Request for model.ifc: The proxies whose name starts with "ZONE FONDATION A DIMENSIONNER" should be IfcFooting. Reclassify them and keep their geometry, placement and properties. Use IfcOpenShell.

First a look at what the model holds.

```python
import re

import ifcopenshell

model = ifcopenshell.open("model.ifc")
print(model.schema)
seen = {}
for e in model.by_type("IfcBuildingElementProxy"):
    name = re.sub(r":\d+(:\d+)?$", "", e.Name or "")  # drop the element id that some exporters append
    seen[name] = seen.get(name, 0) + 1
for name, count in sorted(seen.items()):
    print(count, "x", name)
```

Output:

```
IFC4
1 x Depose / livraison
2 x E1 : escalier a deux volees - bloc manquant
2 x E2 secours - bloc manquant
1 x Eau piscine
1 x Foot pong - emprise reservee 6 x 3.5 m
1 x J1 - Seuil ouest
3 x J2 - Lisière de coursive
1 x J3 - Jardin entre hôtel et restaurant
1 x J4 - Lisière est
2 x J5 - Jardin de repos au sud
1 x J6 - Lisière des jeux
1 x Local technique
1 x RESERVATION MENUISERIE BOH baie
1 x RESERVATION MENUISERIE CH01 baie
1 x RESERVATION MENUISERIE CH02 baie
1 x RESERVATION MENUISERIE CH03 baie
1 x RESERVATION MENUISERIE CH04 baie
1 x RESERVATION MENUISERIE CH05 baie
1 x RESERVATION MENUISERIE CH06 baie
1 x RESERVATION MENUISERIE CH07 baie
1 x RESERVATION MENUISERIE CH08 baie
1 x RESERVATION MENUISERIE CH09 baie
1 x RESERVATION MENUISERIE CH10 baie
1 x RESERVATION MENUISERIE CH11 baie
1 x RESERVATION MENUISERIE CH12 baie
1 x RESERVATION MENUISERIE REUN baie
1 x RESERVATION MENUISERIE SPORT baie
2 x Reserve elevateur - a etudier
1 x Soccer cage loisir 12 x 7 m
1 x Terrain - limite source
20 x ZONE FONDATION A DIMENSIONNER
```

```python
import ifcopenshell
import ifcopenshell.api.root

model = ifcopenshell.open("model.ifc")

proxies = [e.id() for e in model.by_type("IfcBuildingElementProxy") if (e.Name or "").startswith("ZONE FONDATION A DIMENSIONNER")]
for step_id in proxies:
    proxy = model.by_id(step_id)
    ifcopenshell.api.root.reassign_class(model, product=proxy, ifc_class="IfcFooting")

print(sum(model.by_id(i).is_a("IfcFooting") for i in proxies), "reclassified")

model.write("model_updated.ifc")
```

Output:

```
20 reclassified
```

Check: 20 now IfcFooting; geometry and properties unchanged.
